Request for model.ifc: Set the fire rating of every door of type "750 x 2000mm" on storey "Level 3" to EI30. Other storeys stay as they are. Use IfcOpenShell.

First a look at what the model holds.

```python
import ifcopenshell
import ifcopenshell.util.element

model = ifcopenshell.open("model.ifc")
print(model.schema)
storey = next(s for s in model.by_type("IfcBuildingStorey") if s.Name == "Level 3")
doors = [e for e in ifcopenshell.util.element.get_decomposition(storey) if e.is_a("IfcDoor")]
seen = {}
for e in doors:
    element_type = ifcopenshell.util.element.get_type(e)
    key = (element_type.Name if element_type != e and element_type else None, ifcopenshell.util.element.get_pset(e, "Pset_DoorCommon", "FireRating"))
    seen[key] = seen.get(key, 0) + 1
for (name, value), count in sorted(seen.items(), key=str):
    print(count, "x", name, "|", value)
```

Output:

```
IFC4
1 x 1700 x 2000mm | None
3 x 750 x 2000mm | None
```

```python
import ifcopenshell
import ifcopenshell.api.pset
import ifcopenshell.util.element

model = ifcopenshell.open("model.ifc")

storey = next(s for s in model.by_type("IfcBuildingStorey") if s.Name == "Level 3")
doors = [e for e in ifcopenshell.util.element.get_decomposition(storey) if e.is_a("IfcDoor")]

count = 0
for e in doors:
    element_type = ifcopenshell.util.element.get_type(e)
    if element_type in (None, e) or element_type.Name != "750 x 2000mm":
        continue
    # add_pset returns the element's existing set when there is one.
    pset = ifcopenshell.api.pset.add_pset(model, product=e, name="Pset_DoorCommon")
    ifcopenshell.api.pset.edit_pset(model, pset=pset, properties={"FireRating": "EI30"})
    count += 1

print(count, "doors updated")

model.write("model_edited.ifc")
```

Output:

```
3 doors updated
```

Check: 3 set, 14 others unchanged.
